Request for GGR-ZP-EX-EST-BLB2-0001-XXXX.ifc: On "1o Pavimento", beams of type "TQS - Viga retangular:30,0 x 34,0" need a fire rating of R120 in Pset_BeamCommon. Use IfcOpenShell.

First a look at what the model holds.

```python
import ifcopenshell
import ifcopenshell.util.element

model = ifcopenshell.open("GGR-ZP-EX-EST-BLB2-0001-XXXX.ifc")
print(model.schema)
storey = next(s for s in model.by_type("IfcBuildingStorey") if s.Name == "1o Pavimento")
beams = [e for e in ifcopenshell.util.element.get_decomposition(storey) if e.is_a("IfcBeam")]
seen = {}
for e in beams:
    element_type = ifcopenshell.util.element.get_type(e)
    key = (element_type.Name if element_type != e and element_type else None, ifcopenshell.util.element.get_pset(e, "Pset_BeamCommon", "FireRating"))
    seen[key] = seen.get(key, 0) + 1
for (name, value), count in sorted(seen.items(), key=str):
    print(count, "x", name, "|", value)
```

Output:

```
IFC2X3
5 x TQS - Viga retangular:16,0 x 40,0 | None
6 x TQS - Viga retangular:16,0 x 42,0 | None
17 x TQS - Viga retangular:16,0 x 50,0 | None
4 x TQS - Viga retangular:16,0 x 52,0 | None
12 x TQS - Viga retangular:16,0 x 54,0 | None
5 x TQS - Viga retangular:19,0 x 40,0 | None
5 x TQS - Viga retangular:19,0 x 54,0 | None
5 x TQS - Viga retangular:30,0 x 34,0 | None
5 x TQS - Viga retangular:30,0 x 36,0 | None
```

```python
import ifcopenshell
import ifcopenshell.api.pset
import ifcopenshell.util.element

model = ifcopenshell.open("GGR-ZP-EX-EST-BLB2-0001-XXXX.ifc")

storey = next(s for s in model.by_type("IfcBuildingStorey") if s.Name == "1o Pavimento")
beams = [e for e in ifcopenshell.util.element.get_decomposition(storey) if e.is_a("IfcBeam")]

count = 0
for e in beams:
    element_type = ifcopenshell.util.element.get_type(e)
    if element_type in (None, e) or element_type.Name != "TQS - Viga retangular:30,0 x 34,0":
        continue
    # add_pset returns the element's existing set when there is one.
    pset = ifcopenshell.api.pset.add_pset(model, product=e, name="Pset_BeamCommon")
    ifcopenshell.api.pset.edit_pset(model, pset=pset, properties={"FireRating": "R120"})
    count += 1

print(count, "beams updated")

model.write("GGR-ZP-EX-EST-BLB2-0001-XXXX_edited.ifc")
```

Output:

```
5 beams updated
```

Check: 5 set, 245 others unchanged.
